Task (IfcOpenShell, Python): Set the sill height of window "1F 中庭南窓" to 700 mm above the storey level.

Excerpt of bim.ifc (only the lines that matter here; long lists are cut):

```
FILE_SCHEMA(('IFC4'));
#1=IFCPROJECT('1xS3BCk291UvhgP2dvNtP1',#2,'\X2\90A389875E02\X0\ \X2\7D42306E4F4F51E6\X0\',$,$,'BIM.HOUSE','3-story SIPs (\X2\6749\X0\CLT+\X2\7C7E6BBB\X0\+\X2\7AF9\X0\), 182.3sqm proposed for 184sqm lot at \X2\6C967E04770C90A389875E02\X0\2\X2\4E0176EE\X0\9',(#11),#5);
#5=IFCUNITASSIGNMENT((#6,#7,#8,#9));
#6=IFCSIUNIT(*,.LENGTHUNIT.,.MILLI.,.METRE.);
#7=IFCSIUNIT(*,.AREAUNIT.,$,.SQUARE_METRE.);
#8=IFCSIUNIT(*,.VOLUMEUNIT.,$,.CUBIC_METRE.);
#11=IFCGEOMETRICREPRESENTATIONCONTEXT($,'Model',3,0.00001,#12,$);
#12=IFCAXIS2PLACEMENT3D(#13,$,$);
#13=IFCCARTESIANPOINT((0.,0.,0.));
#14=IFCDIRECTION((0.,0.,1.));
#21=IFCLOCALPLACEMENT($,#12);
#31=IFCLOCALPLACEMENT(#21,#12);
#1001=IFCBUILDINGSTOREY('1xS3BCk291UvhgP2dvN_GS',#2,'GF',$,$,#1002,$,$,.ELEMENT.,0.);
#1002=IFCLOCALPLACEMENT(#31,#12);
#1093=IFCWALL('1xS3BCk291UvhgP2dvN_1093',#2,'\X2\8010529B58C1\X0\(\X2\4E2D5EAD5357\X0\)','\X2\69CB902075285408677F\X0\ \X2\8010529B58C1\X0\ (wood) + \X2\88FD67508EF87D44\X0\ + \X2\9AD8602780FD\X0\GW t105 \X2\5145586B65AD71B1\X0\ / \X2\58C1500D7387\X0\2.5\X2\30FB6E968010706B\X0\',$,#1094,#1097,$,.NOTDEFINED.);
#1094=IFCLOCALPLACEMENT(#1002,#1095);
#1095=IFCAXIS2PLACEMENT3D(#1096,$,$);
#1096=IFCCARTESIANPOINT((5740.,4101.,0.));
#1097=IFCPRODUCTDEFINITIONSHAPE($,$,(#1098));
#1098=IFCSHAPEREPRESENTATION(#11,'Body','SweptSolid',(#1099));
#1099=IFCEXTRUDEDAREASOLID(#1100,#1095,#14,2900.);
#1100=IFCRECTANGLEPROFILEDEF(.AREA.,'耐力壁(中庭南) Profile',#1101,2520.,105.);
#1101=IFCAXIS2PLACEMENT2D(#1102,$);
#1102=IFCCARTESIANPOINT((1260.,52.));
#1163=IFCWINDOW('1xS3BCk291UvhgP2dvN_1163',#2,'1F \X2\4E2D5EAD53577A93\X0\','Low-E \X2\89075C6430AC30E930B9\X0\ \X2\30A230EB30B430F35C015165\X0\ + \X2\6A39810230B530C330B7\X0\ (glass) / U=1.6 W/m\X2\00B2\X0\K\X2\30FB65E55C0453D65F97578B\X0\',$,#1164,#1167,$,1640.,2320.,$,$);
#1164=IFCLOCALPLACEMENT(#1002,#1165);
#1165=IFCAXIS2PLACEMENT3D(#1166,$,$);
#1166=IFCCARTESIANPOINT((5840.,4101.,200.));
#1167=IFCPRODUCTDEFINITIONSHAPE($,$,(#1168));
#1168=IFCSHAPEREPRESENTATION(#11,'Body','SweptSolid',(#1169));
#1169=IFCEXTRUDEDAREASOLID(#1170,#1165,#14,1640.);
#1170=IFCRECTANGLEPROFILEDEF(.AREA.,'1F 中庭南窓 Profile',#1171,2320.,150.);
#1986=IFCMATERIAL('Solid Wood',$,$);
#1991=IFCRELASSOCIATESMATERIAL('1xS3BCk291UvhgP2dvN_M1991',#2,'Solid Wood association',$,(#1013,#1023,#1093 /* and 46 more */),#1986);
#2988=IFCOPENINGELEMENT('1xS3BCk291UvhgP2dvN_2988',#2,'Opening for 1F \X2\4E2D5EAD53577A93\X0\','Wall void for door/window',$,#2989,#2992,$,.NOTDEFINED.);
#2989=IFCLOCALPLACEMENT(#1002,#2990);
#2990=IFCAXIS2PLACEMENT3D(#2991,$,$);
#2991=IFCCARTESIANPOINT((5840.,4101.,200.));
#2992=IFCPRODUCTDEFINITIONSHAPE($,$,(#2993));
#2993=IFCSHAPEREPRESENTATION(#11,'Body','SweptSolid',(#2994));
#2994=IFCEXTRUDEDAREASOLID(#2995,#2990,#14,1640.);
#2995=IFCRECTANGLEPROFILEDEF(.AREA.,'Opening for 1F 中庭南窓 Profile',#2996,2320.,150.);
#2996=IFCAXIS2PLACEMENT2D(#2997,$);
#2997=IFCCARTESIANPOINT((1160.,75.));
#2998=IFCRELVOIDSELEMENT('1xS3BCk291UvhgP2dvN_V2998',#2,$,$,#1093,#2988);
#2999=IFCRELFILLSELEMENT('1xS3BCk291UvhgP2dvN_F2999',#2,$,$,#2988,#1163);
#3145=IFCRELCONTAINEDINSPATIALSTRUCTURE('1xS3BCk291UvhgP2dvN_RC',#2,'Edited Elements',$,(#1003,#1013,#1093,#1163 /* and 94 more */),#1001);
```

```python
import numpy as np
import ifcopenshell
import ifcopenshell.api.geometry
import ifcopenshell.geom
import ifcopenshell.util.element
import ifcopenshell.util.placement
import ifcopenshell.util.shape
import ifcopenshell.util.unit

model = ifcopenshell.open("bim.ifc")
unit_scale = ifcopenshell.util.unit.calculate_unit_scale(model)

window = model.by_id(1163)
opening = window.FillsVoids[0].RelatingOpeningElement
storey = ifcopenshell.util.element.get_container(window, ifc_class="IfcBuildingStorey")
level = ifcopenshell.util.placement.get_local_placement(storey.ObjectPlacement)[2, 3]

# The opening's origin need not be at the sill, so measure its lowest point.
shape = ifcopenshell.geom.create_shape(ifcopenshell.geom.settings(), opening)
bottom = ifcopenshell.util.shape.get_shape_bottom_elevation(shape, shape.geometry) / unit_scale
dz = level + 0.7 / unit_scale - bottom

shift = np.array([0.0, 0.0, dz])
# The window is not placed relative to its opening, so move both.
for product in (opening, window):
    matrix = ifcopenshell.util.placement.get_local_placement(product.ObjectPlacement)
    matrix[:3, 3] += shift
    ifcopenshell.api.geometry.edit_object_placement(model, product=product, matrix=matrix, is_si=False)

print(f"moved by {dz * unit_scale:+.3f} m")

model.write("bim_rev.ifc")
```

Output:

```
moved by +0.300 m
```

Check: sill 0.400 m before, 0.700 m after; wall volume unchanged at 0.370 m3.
